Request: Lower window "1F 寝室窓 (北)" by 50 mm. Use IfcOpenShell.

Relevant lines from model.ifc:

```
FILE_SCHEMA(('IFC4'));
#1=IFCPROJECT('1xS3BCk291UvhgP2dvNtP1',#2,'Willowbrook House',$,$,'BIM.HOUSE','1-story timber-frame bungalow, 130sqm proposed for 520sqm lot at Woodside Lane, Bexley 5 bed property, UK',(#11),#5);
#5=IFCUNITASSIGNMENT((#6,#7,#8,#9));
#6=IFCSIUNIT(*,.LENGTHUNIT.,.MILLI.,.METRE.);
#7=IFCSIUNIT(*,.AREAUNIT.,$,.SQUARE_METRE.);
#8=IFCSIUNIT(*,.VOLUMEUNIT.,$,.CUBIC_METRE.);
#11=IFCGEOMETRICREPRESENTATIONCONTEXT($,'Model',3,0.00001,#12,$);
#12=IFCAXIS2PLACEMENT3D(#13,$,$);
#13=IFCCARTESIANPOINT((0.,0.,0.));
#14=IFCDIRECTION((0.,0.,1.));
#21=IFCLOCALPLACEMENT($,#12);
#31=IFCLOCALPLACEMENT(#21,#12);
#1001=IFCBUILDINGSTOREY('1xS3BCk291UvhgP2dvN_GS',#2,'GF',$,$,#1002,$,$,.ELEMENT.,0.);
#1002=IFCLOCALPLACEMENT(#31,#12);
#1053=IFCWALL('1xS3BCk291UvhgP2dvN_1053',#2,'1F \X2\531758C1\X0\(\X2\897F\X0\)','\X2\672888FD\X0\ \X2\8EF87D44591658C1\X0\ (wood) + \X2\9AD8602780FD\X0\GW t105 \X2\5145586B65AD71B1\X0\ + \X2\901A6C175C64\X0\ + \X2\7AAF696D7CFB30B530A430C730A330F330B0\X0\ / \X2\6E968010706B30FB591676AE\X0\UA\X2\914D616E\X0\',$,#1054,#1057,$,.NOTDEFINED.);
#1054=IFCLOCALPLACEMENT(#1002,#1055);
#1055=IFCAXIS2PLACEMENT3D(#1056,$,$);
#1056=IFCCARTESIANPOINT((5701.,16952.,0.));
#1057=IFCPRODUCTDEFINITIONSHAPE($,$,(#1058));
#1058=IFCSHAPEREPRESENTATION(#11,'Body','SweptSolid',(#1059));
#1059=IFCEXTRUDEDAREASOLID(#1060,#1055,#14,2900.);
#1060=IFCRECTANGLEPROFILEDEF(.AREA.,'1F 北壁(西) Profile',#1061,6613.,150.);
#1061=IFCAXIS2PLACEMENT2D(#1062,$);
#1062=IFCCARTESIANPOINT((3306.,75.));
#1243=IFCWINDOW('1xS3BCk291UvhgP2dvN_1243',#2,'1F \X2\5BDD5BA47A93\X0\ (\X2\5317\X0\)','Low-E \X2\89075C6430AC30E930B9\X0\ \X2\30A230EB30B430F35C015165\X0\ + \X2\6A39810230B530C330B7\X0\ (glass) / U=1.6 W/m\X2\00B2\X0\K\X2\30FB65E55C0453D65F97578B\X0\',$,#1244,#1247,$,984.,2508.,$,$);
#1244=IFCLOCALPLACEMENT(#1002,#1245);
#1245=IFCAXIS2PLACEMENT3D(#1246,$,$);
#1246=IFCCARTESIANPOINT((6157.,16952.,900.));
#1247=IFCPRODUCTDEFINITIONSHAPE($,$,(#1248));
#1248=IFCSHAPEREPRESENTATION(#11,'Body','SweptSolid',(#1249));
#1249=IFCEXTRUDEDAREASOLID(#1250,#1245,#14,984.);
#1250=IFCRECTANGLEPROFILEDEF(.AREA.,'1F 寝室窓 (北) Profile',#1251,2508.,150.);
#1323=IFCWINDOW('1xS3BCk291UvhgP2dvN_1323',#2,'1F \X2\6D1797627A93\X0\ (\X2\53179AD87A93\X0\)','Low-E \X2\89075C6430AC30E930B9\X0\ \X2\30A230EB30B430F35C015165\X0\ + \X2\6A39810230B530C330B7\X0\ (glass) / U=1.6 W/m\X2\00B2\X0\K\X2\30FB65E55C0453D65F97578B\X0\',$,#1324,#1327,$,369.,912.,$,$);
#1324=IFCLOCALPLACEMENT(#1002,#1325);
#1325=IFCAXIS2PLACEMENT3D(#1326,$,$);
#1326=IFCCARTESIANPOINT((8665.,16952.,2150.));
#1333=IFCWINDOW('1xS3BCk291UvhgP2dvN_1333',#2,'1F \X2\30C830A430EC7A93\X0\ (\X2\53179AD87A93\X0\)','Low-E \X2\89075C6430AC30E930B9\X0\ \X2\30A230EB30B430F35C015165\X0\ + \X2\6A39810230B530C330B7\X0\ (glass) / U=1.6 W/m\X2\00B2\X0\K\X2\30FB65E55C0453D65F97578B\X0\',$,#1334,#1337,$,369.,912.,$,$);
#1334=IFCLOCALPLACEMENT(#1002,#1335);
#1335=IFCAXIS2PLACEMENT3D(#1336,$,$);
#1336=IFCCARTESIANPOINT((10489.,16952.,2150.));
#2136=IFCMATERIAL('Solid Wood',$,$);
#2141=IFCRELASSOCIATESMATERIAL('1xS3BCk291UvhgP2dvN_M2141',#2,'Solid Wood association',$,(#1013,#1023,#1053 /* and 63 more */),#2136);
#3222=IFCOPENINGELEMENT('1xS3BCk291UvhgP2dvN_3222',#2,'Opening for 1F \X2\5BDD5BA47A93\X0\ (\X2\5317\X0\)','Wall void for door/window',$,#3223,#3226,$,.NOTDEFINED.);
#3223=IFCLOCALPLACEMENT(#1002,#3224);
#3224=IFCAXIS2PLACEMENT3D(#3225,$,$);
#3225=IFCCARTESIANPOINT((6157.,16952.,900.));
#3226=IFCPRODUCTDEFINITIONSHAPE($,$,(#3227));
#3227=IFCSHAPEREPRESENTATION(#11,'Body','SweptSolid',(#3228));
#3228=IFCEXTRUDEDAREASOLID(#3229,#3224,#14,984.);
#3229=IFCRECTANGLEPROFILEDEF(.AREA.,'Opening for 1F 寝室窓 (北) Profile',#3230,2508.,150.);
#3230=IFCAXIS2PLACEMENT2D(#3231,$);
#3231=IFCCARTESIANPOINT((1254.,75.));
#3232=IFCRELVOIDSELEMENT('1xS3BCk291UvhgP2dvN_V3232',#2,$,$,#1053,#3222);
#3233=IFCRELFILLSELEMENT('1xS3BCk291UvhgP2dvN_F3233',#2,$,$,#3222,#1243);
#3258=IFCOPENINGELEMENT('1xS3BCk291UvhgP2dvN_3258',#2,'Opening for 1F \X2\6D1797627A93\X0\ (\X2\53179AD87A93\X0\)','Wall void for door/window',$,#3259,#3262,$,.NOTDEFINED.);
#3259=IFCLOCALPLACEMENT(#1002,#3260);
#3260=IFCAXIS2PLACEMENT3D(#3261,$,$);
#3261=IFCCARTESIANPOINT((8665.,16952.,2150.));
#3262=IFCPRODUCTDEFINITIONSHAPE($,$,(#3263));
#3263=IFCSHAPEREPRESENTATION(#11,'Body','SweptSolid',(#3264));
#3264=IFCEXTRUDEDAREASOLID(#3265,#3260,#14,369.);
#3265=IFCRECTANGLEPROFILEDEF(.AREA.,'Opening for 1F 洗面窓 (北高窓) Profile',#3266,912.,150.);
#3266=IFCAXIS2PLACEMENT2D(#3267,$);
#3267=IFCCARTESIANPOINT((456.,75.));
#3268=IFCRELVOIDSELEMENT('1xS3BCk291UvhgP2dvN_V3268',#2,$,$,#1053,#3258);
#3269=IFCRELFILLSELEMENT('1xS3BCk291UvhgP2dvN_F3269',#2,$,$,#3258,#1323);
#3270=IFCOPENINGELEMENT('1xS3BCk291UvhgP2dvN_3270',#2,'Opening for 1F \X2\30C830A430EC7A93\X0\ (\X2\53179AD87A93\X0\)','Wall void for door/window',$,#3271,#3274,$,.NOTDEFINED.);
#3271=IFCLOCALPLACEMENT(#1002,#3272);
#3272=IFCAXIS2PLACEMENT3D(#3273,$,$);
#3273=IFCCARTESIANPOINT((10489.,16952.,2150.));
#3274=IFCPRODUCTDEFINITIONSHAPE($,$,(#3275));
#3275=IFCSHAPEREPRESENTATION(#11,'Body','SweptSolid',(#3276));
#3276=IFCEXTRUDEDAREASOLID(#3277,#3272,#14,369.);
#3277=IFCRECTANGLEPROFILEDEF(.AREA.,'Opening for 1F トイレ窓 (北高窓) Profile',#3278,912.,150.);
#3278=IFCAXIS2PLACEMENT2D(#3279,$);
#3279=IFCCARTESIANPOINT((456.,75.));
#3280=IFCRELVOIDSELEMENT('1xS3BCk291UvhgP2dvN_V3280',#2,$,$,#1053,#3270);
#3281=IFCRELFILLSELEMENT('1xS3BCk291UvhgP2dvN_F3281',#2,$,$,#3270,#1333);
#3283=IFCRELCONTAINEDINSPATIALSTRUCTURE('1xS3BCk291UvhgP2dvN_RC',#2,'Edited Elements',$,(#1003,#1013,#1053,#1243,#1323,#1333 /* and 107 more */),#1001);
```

```python
import numpy as np
import ifcopenshell
import ifcopenshell.api.geometry
import ifcopenshell.util.placement
import ifcopenshell.util.unit

model = ifcopenshell.open("model.ifc")
unit_scale = ifcopenshell.util.unit.calculate_unit_scale(model)

window = model.by_guid("1xS3BCk291UvhgP2dvN_1243")
opening = window.FillsVoids[0].RelatingOpeningElement
dz = -0.05 / unit_scale

shift = np.array([0.0, 0.0, dz])
# The window is not placed relative to its opening, so move both.
for product in (opening, window):
    matrix = ifcopenshell.util.placement.get_local_placement(product.ObjectPlacement)
    matrix[:3, 3] += shift
    ifcopenshell.api.geometry.edit_object_placement(model, product=product, matrix=matrix, is_si=False)

print(f"moved by {dz * unit_scale:+.3f} m")

model.write("model-out.ifc")
```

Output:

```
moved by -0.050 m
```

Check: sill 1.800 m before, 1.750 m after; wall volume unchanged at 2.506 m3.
